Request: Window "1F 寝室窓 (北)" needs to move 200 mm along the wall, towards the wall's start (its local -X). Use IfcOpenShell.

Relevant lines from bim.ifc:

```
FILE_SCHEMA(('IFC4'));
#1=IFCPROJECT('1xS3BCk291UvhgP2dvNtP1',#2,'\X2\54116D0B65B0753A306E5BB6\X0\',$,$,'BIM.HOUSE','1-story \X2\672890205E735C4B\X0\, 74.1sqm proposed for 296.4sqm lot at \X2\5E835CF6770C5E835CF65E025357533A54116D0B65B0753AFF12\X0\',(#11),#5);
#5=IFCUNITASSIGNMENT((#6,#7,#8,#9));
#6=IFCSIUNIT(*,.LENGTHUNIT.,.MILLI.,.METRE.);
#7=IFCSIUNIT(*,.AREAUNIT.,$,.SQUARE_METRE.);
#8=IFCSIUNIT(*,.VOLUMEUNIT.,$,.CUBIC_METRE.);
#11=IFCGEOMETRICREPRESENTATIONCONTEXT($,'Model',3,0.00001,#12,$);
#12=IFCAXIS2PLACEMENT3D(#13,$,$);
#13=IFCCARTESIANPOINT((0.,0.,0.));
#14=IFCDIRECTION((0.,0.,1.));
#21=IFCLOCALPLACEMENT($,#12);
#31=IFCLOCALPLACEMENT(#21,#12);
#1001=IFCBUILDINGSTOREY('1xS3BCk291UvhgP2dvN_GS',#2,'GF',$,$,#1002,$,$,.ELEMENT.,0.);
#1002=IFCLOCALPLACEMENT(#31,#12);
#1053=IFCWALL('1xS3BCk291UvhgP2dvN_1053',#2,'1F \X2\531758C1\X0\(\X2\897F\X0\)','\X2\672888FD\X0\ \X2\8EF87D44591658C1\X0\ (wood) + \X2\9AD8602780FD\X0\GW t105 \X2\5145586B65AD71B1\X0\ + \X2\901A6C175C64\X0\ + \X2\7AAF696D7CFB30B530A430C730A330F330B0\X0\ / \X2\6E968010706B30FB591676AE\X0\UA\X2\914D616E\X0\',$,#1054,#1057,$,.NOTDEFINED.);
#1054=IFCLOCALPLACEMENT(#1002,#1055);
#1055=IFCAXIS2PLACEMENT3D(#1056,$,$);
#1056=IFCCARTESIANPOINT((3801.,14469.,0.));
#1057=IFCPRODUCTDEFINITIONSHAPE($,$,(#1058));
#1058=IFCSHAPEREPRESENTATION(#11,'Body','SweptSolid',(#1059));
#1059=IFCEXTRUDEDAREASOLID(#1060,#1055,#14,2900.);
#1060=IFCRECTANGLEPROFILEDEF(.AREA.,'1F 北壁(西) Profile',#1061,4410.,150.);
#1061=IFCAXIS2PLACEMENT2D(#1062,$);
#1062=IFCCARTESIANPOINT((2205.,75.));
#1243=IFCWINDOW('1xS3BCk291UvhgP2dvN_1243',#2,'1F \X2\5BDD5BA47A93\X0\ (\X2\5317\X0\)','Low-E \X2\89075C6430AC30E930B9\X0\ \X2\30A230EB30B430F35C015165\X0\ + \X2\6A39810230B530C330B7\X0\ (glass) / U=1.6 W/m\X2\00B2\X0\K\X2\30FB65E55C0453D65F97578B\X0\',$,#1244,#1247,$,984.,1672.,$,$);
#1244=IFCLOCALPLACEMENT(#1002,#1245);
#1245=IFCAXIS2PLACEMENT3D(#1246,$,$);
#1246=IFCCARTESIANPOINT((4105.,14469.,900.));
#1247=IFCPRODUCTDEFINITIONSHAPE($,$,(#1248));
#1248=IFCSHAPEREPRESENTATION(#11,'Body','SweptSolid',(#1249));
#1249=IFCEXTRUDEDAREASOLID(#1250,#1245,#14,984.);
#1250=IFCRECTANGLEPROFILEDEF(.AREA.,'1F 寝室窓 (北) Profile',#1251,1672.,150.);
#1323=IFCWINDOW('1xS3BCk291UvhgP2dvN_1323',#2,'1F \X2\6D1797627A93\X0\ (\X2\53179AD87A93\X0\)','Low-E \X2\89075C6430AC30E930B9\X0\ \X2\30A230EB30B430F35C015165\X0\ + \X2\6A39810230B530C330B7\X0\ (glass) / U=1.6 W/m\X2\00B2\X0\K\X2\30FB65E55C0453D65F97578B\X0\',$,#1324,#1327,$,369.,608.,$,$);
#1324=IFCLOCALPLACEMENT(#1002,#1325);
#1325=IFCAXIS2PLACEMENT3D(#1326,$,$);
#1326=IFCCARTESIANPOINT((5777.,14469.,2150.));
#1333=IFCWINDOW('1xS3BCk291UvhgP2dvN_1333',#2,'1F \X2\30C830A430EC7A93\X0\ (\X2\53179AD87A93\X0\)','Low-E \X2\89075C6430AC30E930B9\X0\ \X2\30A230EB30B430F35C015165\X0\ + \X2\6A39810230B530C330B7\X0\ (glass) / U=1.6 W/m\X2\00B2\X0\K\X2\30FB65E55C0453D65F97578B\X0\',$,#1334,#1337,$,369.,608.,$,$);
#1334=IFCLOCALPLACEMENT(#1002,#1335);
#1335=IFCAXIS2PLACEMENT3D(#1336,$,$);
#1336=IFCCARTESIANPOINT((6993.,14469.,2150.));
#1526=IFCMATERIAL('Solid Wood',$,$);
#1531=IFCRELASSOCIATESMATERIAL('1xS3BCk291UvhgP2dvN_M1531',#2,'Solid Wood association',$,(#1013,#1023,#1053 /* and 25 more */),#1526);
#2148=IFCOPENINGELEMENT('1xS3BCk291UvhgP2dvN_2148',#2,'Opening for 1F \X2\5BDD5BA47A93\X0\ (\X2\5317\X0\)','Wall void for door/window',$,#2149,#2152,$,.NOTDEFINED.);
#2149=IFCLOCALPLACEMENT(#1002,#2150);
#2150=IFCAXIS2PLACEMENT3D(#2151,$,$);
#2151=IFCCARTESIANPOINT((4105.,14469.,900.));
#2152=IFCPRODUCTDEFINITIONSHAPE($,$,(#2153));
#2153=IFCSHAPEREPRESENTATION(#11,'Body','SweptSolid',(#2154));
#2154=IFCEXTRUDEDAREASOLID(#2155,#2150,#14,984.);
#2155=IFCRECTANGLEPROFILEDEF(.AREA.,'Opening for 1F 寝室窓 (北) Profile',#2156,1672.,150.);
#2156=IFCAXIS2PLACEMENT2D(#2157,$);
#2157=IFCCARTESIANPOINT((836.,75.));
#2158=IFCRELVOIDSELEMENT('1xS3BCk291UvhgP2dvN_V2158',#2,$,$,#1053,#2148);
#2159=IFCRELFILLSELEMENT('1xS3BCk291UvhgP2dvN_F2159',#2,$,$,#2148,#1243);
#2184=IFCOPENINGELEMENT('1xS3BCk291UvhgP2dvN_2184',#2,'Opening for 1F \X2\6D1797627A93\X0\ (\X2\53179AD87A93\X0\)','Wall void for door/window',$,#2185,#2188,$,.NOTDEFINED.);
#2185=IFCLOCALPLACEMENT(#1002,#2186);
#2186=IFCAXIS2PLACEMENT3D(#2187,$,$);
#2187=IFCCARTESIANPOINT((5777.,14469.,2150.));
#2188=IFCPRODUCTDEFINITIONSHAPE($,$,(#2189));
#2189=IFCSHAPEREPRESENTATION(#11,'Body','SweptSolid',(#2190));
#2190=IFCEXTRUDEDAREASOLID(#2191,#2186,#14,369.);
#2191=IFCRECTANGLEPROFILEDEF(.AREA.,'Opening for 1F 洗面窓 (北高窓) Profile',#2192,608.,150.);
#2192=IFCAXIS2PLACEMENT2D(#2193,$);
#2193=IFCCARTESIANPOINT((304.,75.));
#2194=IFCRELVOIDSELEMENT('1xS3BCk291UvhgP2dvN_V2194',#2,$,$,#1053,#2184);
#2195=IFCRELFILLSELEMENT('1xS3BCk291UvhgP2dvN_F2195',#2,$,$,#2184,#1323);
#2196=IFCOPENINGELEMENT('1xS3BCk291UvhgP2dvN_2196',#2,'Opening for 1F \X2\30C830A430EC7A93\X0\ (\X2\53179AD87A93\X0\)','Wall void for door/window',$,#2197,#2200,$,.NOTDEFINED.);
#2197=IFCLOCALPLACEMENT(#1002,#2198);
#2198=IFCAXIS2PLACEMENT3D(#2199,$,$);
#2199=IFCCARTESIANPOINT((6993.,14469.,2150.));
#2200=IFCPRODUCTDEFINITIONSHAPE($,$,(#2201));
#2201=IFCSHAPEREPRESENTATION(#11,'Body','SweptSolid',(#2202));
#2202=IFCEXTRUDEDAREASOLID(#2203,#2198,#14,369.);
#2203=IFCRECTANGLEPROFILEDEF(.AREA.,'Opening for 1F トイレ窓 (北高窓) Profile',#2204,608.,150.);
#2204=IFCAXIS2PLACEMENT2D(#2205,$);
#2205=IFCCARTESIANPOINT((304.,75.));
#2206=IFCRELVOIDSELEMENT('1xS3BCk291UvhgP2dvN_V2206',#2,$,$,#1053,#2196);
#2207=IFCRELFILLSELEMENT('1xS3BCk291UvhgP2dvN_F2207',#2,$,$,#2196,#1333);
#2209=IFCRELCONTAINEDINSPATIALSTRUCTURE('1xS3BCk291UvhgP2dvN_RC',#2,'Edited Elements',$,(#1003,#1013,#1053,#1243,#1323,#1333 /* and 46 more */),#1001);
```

```python
import ifcopenshell
import ifcopenshell.api.geometry
import ifcopenshell.util.placement
import ifcopenshell.util.unit

model = ifcopenshell.open("bim.ifc")
unit_scale = ifcopenshell.util.unit.calculate_unit_scale(model)

window = model.by_guid("1xS3BCk291UvhgP2dvN_1243")
opening = window.FillsVoids[0].RelatingOpeningElement
wall = opening.VoidsElements[0].RelatingBuildingElement

wall_matrix = ifcopenshell.util.placement.get_local_placement(wall.ObjectPlacement)
shift = wall_matrix[:3, 0] * -0.2 / unit_scale
before = ifcopenshell.util.placement.get_local_placement(window.ObjectPlacement)[:3, 3].copy()

# The window is not placed relative to its opening, so move both.
for product in (opening, window):
    matrix = ifcopenshell.util.placement.get_local_placement(product.ObjectPlacement)
    matrix[:3, 3] += shift
    ifcopenshell.api.geometry.edit_object_placement(model, product=product, matrix=matrix, is_si=False)

after = ifcopenshell.util.placement.get_local_placement(window.ObjectPlacement)[:3, 3]
print("window moved by", (after - before).round(3) + 0.0)

model.write("bim-out.ifc")
```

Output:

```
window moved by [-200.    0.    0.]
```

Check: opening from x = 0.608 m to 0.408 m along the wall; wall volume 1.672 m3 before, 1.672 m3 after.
